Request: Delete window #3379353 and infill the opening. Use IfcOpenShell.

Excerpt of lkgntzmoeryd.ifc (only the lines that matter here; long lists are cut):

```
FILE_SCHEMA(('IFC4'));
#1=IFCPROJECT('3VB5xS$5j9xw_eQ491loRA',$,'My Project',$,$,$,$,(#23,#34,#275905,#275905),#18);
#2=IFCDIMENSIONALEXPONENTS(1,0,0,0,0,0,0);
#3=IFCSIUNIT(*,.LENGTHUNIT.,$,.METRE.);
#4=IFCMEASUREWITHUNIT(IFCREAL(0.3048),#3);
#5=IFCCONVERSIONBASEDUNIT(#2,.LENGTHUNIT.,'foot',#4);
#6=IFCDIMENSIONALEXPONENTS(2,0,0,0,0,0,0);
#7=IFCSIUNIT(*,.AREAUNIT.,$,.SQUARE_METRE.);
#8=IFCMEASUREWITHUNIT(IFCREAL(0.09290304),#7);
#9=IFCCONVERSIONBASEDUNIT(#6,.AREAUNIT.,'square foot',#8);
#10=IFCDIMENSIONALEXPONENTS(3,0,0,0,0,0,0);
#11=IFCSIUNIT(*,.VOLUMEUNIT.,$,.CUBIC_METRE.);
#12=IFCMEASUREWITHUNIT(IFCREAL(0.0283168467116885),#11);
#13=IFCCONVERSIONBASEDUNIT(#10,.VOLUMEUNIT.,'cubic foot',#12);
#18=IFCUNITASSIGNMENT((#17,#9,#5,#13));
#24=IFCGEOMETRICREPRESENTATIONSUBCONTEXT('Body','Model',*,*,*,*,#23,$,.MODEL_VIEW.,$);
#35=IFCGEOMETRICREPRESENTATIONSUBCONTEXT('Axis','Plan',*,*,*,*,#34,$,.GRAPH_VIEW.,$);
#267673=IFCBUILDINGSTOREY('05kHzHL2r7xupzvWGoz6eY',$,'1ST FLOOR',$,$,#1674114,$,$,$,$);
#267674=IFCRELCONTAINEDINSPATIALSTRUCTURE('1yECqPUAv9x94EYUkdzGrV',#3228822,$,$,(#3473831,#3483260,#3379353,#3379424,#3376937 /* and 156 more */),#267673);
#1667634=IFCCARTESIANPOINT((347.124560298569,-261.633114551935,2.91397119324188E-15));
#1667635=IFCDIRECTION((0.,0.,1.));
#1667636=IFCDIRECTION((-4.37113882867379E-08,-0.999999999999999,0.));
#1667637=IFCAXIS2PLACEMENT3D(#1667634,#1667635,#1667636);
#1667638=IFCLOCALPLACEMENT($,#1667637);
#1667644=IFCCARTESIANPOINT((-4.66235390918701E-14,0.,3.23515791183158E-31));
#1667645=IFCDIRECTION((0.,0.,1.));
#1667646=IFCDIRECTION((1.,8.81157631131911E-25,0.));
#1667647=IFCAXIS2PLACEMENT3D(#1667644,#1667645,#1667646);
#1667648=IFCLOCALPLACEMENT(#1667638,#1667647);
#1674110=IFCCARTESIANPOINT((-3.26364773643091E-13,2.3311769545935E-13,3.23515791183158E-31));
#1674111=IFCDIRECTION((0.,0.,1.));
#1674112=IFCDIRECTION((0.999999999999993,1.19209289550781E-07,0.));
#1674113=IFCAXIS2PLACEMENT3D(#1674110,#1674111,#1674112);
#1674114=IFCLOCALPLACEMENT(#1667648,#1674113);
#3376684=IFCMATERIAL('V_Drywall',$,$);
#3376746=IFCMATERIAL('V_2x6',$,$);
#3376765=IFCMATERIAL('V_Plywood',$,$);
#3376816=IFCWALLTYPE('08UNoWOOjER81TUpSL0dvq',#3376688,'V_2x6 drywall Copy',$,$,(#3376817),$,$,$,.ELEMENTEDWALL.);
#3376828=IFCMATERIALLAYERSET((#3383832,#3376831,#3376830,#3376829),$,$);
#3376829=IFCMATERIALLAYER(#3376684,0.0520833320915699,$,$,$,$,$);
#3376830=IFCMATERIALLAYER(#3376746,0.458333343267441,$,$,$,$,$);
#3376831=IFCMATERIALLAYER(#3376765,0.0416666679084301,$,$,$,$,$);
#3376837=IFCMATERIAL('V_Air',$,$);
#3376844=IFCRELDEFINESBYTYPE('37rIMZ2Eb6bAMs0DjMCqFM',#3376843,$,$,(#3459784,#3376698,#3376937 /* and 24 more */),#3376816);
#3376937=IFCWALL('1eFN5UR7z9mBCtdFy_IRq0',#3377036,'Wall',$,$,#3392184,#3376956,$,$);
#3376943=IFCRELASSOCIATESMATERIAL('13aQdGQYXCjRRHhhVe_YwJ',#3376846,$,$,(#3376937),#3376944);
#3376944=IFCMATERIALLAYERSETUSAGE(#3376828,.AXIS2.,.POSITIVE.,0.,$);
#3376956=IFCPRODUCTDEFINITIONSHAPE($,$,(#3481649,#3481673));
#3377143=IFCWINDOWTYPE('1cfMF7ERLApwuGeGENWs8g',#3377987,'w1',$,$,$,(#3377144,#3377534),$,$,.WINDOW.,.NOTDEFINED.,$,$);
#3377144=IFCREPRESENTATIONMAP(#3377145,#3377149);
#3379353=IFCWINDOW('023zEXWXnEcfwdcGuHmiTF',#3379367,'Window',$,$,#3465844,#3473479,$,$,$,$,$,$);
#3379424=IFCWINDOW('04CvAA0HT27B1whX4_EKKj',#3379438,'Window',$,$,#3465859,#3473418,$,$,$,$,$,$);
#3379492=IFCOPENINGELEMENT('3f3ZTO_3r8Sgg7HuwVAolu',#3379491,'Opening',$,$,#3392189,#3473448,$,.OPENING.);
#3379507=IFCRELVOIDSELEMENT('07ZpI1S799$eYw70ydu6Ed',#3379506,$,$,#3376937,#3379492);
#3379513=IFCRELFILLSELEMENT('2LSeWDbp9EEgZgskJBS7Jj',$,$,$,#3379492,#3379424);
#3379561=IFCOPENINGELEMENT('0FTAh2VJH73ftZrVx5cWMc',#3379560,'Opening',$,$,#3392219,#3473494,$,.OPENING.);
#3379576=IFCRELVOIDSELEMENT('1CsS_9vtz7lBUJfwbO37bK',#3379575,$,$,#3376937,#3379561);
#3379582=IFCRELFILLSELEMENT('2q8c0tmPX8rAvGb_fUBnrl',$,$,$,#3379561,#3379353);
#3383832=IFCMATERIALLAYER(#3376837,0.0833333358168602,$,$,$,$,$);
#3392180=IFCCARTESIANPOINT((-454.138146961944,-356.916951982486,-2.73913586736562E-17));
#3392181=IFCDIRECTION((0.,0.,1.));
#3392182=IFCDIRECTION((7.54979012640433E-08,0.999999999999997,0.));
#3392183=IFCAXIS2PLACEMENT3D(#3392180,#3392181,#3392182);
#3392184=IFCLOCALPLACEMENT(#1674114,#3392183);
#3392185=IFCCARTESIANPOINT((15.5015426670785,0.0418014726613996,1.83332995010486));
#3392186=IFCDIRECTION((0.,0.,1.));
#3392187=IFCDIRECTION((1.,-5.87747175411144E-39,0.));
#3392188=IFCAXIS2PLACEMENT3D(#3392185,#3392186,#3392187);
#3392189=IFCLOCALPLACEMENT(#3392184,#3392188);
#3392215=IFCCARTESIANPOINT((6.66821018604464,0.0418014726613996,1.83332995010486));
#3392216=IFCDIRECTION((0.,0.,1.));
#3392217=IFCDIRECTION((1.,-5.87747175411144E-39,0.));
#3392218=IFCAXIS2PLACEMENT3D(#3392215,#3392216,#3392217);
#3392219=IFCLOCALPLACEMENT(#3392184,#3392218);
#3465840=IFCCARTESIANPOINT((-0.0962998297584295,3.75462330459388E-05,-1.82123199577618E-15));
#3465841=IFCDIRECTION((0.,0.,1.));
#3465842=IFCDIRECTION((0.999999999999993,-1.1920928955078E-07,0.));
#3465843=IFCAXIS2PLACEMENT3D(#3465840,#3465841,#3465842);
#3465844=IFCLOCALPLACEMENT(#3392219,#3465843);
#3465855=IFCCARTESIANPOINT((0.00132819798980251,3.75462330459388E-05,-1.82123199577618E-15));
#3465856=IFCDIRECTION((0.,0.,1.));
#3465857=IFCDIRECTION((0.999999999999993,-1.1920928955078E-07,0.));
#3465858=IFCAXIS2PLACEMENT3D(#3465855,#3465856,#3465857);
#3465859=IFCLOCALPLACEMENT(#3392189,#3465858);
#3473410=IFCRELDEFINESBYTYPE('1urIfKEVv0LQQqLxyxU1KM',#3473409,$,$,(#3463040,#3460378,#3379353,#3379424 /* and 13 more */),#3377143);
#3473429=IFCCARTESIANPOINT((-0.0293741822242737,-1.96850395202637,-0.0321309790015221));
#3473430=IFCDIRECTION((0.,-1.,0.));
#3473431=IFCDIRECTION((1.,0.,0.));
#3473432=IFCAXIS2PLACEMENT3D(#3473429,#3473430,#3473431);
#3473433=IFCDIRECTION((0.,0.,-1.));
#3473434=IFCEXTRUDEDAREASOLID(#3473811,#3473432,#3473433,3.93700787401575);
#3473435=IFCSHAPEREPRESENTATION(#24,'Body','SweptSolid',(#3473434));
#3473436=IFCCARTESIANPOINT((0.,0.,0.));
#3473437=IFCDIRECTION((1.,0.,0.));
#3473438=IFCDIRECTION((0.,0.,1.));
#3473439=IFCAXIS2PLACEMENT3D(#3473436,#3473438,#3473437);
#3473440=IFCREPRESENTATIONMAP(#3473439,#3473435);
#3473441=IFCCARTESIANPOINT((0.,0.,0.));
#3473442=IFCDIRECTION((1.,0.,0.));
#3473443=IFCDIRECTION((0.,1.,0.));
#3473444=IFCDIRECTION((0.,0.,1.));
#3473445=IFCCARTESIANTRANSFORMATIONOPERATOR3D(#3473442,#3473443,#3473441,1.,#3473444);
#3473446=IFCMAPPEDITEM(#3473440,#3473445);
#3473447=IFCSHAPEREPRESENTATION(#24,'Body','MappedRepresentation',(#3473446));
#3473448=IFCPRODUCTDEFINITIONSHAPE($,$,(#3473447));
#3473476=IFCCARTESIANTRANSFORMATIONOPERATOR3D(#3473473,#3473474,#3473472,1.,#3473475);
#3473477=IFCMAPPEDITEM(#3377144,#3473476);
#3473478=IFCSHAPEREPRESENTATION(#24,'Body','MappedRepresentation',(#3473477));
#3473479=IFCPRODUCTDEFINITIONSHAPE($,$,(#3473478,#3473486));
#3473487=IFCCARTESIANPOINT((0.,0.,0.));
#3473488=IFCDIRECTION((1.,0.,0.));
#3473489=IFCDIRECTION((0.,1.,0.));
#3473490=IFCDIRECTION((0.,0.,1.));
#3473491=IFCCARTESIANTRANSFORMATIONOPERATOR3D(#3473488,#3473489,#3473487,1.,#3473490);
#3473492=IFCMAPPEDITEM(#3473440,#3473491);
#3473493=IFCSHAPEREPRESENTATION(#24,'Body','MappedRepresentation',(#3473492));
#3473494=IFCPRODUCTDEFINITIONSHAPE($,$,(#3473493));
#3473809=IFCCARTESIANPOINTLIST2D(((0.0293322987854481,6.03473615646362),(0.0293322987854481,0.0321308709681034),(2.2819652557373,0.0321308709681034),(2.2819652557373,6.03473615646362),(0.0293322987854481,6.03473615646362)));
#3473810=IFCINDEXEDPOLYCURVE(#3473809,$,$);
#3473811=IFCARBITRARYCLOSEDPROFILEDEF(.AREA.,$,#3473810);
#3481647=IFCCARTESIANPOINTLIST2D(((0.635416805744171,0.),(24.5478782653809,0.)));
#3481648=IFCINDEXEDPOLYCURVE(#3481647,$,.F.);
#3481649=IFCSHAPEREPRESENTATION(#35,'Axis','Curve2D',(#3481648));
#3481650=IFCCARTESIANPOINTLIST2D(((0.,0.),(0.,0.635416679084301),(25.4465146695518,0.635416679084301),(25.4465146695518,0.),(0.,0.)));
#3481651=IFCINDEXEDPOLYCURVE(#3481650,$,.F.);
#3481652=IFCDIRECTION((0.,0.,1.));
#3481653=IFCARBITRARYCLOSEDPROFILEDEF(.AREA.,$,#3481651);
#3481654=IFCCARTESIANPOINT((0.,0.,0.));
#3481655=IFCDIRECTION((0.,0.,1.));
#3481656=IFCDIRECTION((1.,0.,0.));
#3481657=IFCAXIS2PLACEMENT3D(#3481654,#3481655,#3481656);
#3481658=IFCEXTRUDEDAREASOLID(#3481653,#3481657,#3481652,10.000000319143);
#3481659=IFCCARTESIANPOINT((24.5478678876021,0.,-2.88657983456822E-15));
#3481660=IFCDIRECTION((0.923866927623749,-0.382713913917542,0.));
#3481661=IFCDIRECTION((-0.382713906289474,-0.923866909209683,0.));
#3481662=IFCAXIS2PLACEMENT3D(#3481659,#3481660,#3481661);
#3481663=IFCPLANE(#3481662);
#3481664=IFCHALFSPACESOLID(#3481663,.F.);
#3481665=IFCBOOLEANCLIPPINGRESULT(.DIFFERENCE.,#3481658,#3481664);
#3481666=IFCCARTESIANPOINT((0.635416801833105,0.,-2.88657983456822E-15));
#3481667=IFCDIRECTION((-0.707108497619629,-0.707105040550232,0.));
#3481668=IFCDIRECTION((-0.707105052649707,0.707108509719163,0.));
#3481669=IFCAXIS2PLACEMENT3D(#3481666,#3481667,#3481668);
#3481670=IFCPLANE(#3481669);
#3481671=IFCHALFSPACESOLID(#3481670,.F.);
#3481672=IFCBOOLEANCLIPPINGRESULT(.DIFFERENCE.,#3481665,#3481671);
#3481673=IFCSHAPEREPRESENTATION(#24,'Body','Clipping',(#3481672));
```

```python
import ifcopenshell
import ifcopenshell.api.feature
import ifcopenshell.api.root
import ifcopenshell.geom
import ifcopenshell.util.shape

model = ifcopenshell.open("lkgntzmoeryd.ifc")
settings = ifcopenshell.geom.settings()


def volume(element):
    """Net volume in cubic metres, openings subtracted."""
    shape = ifcopenshell.geom.create_shape(settings, element)
    return ifcopenshell.util.shape.get_volume(shape.geometry)


window = model.by_guid("023zEXWXnEcfwdcGuHmiTF")
opening = window.FillsVoids[0].RelatingOpeningElement
wall = opening.VoidsElements[0].RelatingBuildingElement
before = volume(wall)

ifcopenshell.api.root.remove_product(model, product=window)
ifcopenshell.api.feature.remove_feature(model, feature=opening)

after = volume(wall)

print(f"wall volume {before:.3f} -> {after:.3f} m3")

model.write("lkgntzmoeryd_edited.ifc")
```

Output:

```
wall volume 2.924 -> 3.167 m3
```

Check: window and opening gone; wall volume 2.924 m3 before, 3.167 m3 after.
